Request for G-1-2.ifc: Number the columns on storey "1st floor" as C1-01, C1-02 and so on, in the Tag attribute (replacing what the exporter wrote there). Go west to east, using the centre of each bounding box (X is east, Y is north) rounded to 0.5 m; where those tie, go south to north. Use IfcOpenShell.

First a look at what the model holds.

```python
import ifcopenshell
import ifcopenshell.util.element
import ifcopenshell.util.placement

model = ifcopenshell.open("G-1-2.ifc")
print(model.schema)
storey = next(s for s in model.by_type("IfcBuildingStorey") if s.Name == "1st floor")
columns = [e for e in ifcopenshell.util.element.get_decomposition(storey) if e.is_a("IfcColumn")]
for e in sorted(columns, key=lambda e: e.id()):
    origin = ifcopenshell.util.placement.get_local_placement(e.ObjectPlacement)[:3, 3]
    print(e.id(), e.Tag, e.Name, origin.round(2) + 0.0, sep=" | ")
```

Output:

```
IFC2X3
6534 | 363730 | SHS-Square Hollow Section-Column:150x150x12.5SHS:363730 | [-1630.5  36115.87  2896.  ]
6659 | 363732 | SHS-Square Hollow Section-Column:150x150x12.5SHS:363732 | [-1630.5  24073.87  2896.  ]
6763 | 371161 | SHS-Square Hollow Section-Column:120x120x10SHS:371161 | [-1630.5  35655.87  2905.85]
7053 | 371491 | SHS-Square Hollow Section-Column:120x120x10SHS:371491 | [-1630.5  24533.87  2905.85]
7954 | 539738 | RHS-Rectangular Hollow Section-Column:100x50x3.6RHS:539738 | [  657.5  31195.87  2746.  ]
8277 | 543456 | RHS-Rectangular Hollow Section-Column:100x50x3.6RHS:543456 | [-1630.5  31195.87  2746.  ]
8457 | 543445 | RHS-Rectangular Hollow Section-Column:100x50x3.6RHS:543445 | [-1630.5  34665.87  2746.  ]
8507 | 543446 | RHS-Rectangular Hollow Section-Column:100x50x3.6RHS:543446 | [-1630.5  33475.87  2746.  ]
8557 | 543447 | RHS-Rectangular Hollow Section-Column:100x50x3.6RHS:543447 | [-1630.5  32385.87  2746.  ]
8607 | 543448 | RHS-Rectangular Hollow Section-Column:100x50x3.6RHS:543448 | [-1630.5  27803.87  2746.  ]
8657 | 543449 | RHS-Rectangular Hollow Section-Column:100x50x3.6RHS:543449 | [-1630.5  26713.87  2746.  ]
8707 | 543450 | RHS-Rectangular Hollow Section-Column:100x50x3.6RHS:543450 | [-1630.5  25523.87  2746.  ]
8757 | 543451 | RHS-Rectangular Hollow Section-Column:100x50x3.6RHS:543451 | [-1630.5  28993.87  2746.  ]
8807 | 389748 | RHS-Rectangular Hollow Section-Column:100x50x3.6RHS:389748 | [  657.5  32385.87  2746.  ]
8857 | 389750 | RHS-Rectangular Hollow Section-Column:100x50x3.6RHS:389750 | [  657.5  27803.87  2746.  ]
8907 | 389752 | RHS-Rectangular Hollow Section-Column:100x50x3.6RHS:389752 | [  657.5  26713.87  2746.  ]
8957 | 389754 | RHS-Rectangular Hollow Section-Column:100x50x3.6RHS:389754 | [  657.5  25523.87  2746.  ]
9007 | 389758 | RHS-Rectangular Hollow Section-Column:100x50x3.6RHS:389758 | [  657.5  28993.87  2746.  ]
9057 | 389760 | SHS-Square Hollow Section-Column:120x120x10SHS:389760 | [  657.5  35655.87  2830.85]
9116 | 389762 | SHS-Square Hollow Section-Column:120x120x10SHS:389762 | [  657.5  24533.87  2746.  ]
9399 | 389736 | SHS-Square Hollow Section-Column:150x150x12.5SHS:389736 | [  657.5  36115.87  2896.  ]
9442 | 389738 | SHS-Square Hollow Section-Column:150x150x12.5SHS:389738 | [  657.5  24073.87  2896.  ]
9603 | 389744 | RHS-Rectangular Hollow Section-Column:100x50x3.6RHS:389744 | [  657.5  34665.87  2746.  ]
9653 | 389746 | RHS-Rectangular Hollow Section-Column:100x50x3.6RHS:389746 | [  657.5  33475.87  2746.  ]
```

```python
import ifcopenshell
import ifcopenshell.geom
import ifcopenshell.util.element
import ifcopenshell.util.shape

model = ifcopenshell.open("G-1-2.ifc")
settings = ifcopenshell.geom.settings()
settings.set("use-world-coords", True)


def centre(element):
    shape = ifcopenshell.geom.create_shape(settings, element)
    return ifcopenshell.util.shape.get_bbox_centroid(shape.geometry)


storey = next(s for s in model.by_type("IfcBuildingStorey") if s.Name == "1st floor")
columns = [e for e in ifcopenshell.util.element.get_decomposition(storey) if e.is_a("IfcColumn")]

# Insertion points can sit at a corner or the storey origin, so sort by the geometry (in metres).
centres = {e: centre(e) for e in columns}
columns.sort(key=lambda e: (round(centres[e][0] / 0.5), centres[e][1]))

for i, e in enumerate(columns, start=1):
    number = f"C1-{i:02d}"
    e.Tag = number
    print(e.id(), number)

model.write("G-1-2-out.ifc")
```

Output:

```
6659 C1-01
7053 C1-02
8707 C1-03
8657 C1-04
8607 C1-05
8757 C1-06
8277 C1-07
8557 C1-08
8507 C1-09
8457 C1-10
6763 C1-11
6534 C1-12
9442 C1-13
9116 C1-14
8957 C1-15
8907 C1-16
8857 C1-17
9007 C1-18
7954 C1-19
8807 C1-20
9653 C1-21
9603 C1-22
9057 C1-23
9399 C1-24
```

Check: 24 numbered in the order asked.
